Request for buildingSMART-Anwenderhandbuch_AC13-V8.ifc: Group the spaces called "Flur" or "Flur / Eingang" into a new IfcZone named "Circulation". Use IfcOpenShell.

First a look at what the model holds.

```python
import ifcopenshell

model = ifcopenshell.open("buildingSMART-Anwenderhandbuch_AC13-V8.ifc")
print(model.schema)
seen = {}
for space in model.by_type("IfcSpace"):
    seen[space.LongName] = seen.get(space.LongName, 0) + 1
for name, count in sorted(seen.items(), key=str):
    print(count, "x", name)
print("zones:", [z.Name for z in model.by_type("IfcZone")][:20])
```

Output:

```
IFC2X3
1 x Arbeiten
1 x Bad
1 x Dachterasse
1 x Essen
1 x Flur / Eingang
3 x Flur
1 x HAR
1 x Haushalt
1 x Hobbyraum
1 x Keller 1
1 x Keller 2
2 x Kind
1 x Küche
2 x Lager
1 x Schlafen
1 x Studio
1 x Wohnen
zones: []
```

```python
import ifcopenshell
import ifcopenshell.api.group
import ifcopenshell.api.root

model = ifcopenshell.open("buildingSMART-Anwenderhandbuch_AC13-V8.ifc")

names = {"Flur", "Flur / Eingang"}
spaces = [s for s in model.by_type("IfcSpace") if s.LongName in names]

zone = ifcopenshell.api.root.create_entity(model, ifc_class="IfcZone", name="Circulation")
ifcopenshell.api.group.assign_group(model, products=spaces, group=zone)
print(len(spaces), "spaces in", zone.Name)

model.write("buildingSMART-Anwenderhandbuch_AC13-V8_updated.ifc")
```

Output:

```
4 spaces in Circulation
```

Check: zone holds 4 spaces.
